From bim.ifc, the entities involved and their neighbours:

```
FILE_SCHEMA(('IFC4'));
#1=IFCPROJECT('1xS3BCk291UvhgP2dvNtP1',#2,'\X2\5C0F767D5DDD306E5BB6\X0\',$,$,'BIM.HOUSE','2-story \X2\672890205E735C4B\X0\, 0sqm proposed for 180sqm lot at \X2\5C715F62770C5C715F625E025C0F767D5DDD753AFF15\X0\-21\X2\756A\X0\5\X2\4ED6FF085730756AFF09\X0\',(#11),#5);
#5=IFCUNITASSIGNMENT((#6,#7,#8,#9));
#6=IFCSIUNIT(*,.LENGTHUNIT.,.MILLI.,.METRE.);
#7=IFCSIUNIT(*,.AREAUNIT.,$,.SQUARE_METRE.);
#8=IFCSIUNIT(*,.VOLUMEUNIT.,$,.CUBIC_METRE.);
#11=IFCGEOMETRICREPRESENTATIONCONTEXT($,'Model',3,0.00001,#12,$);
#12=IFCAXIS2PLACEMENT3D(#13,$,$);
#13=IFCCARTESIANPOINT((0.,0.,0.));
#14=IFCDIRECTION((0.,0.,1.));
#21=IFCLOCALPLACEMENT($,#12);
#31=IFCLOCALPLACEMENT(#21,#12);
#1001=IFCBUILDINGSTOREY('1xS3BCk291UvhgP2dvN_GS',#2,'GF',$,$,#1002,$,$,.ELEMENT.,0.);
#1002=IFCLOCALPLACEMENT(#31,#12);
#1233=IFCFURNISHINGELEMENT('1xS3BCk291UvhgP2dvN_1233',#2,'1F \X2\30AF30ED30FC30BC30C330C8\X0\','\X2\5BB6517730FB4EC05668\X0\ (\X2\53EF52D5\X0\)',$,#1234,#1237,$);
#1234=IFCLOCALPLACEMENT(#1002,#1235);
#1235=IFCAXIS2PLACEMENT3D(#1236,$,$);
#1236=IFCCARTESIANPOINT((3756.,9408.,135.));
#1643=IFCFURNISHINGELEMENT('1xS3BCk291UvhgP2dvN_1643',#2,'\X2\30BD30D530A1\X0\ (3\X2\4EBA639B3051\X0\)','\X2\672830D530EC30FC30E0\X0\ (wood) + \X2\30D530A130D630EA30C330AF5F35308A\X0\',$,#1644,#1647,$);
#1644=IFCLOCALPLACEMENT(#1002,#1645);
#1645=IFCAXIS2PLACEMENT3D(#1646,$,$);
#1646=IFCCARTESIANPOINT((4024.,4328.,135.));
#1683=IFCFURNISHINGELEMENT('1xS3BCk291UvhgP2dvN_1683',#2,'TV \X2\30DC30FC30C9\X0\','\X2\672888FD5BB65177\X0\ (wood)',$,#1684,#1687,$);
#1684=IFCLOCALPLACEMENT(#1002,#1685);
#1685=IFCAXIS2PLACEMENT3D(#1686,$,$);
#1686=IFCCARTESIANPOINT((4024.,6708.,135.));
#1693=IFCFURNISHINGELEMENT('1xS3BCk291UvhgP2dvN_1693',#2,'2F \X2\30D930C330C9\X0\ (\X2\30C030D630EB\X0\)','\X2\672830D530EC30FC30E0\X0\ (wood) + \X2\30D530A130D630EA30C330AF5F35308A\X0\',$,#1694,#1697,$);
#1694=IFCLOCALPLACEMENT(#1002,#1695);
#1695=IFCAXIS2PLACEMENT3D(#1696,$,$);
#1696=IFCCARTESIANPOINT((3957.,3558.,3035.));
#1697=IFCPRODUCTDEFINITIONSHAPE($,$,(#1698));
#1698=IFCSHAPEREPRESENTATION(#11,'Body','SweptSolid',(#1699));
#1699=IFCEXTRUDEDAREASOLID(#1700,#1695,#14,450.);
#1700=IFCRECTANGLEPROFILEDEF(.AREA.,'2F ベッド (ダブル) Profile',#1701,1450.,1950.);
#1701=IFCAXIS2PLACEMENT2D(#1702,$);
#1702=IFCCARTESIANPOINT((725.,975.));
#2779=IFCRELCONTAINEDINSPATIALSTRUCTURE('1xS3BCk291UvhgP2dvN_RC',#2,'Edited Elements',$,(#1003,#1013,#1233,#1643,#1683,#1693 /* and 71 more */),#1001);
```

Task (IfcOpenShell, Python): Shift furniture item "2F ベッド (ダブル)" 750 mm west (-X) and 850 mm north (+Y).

```python
import ifcopenshell
import ifcopenshell.api.geometry
import ifcopenshell.util.placement

model = ifcopenshell.open("bim.ifc")

item = model.by_guid("1xS3BCk291UvhgP2dvN_1693")
matrix = ifcopenshell.util.placement.get_local_placement(item.ObjectPlacement)
matrix[0, 3] -= 750.0
matrix[1, 3] += 850.0
ifcopenshell.api.geometry.edit_object_placement(model, product=item, matrix=matrix, is_si=False)

print(ifcopenshell.util.placement.get_local_placement(item.ObjectPlacement).round(3) + 0.0)

model.write("bim_rev.ifc")
```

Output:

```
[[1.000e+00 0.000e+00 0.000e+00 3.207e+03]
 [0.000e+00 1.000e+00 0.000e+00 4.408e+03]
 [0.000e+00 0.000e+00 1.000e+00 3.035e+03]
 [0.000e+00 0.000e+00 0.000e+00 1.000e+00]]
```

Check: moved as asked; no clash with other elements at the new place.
